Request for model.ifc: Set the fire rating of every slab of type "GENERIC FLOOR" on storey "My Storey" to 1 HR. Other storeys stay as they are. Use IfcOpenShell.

First a look at what the model holds.

```python
import ifcopenshell
import ifcopenshell.util.element

model = ifcopenshell.open("model.ifc")
print(model.schema)
storey = next(s for s in model.by_type("IfcBuildingStorey") if s.Name == "My Storey")
slabs = [e for e in ifcopenshell.util.element.get_decomposition(storey) if e.is_a("IfcSlab")]
seen = {}
for e in slabs:
    element_type = ifcopenshell.util.element.get_type(e)
    key = (element_type.Name if element_type != e and element_type else None, ifcopenshell.util.element.get_pset(e, "Pset_SlabCommon", "FireRating"))
    seen[key] = seen.get(key, 0) + 1
for (name, value), count in sorted(seen.items(), key=str):
    print(count, "x", name, "|", value)
```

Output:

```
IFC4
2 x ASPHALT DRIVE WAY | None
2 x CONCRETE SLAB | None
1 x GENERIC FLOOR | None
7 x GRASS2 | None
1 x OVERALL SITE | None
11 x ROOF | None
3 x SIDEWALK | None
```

```python
import ifcopenshell
import ifcopenshell.api.pset
import ifcopenshell.util.element

model = ifcopenshell.open("model.ifc")

storey = next(s for s in model.by_type("IfcBuildingStorey") if s.Name == "My Storey")
slabs = [e for e in ifcopenshell.util.element.get_decomposition(storey) if e.is_a("IfcSlab")]

count = 0
for e in slabs:
    element_type = ifcopenshell.util.element.get_type(e)
    if element_type in (None, e) or element_type.Name != "GENERIC FLOOR":
        continue
    # add_pset returns the element's existing set when there is one.
    pset = ifcopenshell.api.pset.add_pset(model, product=e, name="Pset_SlabCommon")
    ifcopenshell.api.pset.edit_pset(model, pset=pset, properties={"FireRating": "1 HR"})
    count += 1

print(count, "slabs updated")

model.write("model_updated.ifc")
```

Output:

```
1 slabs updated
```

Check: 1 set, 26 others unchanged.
